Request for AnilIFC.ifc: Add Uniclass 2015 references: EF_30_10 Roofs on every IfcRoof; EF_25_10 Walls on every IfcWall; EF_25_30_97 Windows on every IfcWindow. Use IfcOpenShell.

First a look at what the model holds.

```python
import ifcopenshell

model = ifcopenshell.open("AnilIFC.ifc")
print(model.schema)
print("classifications:", [c.Name for c in model.by_type("IfcClassification")])
for ifc_class in ("IfcDoor", "IfcRoof", "IfcStair", "IfcWall", "IfcWindow"):
    print(ifc_class, len(model.by_type(ifc_class)))
```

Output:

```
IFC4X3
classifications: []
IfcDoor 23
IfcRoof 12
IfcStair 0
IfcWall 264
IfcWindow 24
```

```python
import ifcopenshell
import ifcopenshell.api.classification

model = ifcopenshell.open("AnilIFC.ifc")

system = ifcopenshell.api.classification.add_classification(model, classification="Uniclass 2015")

codes = {
    "IfcRoof": ("EF_30_10", "Roofs"),
    "IfcWall": ("EF_25_10", "Walls"),
    "IfcWindow": ("EF_25_30_97", "Windows"),
}
for ifc_class, (code, name) in codes.items():
    products = model.by_type(ifc_class)
    ifcopenshell.api.classification.add_reference(
        model, products=products, classification=system, identification=code, name=name
    )
    print(code, len(products))

model.write("AnilIFC_v2.ifc")
```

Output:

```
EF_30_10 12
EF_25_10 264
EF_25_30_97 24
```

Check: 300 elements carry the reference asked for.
